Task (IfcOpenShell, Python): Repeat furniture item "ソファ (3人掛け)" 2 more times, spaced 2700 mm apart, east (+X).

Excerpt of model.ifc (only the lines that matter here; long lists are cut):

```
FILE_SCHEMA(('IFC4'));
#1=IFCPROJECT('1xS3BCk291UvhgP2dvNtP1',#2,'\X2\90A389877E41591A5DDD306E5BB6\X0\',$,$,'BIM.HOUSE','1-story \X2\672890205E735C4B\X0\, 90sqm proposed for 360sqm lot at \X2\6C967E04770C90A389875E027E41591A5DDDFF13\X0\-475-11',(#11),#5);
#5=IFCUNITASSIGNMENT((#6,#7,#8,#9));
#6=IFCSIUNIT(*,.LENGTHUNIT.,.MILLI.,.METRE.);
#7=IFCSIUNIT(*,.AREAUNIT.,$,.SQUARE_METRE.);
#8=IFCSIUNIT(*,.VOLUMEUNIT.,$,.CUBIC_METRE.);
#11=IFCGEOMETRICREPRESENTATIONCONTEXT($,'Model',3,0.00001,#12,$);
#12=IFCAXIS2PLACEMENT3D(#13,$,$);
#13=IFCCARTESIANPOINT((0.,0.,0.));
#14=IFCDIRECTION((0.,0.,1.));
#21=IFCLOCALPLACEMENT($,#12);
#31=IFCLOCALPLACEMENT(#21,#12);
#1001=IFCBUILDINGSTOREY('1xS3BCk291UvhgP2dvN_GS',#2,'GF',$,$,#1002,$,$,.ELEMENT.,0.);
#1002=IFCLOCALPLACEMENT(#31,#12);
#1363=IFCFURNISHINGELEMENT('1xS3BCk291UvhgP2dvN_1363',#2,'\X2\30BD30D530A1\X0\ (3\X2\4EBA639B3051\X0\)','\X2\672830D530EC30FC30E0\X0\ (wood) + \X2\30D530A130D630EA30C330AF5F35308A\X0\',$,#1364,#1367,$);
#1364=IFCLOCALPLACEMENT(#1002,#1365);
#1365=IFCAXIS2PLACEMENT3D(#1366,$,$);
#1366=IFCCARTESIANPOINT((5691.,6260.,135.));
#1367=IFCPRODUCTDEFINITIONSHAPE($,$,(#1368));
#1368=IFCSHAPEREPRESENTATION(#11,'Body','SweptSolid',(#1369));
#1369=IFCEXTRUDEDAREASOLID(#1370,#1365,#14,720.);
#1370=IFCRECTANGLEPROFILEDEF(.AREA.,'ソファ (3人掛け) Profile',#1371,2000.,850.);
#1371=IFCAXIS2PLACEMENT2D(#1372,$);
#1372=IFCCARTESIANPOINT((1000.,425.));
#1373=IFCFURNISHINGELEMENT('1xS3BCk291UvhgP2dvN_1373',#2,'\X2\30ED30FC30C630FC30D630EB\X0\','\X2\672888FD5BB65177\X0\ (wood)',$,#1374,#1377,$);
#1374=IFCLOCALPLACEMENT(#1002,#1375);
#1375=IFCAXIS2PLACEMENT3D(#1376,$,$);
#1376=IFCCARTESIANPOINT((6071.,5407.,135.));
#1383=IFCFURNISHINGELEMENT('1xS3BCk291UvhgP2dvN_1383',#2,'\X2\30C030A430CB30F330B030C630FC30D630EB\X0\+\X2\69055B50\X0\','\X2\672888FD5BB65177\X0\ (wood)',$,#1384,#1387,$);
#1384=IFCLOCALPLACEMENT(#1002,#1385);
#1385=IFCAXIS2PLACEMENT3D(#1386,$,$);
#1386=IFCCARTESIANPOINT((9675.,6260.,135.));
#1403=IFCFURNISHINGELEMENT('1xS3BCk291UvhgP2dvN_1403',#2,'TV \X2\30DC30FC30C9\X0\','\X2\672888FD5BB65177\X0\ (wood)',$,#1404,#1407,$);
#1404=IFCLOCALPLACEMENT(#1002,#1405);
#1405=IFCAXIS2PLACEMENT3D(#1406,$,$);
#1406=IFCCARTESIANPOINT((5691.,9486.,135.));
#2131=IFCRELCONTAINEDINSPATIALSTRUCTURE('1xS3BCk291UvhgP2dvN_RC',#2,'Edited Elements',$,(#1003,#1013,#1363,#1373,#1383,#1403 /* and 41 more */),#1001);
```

```python
import numpy as np
import ifcopenshell
import ifcopenshell.api.geometry
import ifcopenshell.api.root
import ifcopenshell.util.element
import ifcopenshell.util.placement

model = ifcopenshell.open("model.ifc")


def reuse_history(source, copy):
    """copy_class also copies each property set's owner history, people and application; keep the originals."""
    for rel in copy.IsDefinedBy:
        if rel.is_a("IfcRelDefinesByProperties") and (history := rel.RelatingPropertyDefinition.OwnerHistory):
            rel.RelatingPropertyDefinition.OwnerHistory = source.OwnerHistory
            ifcopenshell.util.element.remove_deep2(model, history)


source = model.by_guid("1xS3BCk291UvhgP2dvN_1363")
base = ifcopenshell.util.placement.get_local_placement(source.ObjectPlacement)
step = np.array([1.0, 0.0, 0.0]) * 2700.0

for i in range(1, 3):
    copy = ifcopenshell.api.root.copy_class(model, product=source)
    copy.Representation = ifcopenshell.util.element.copy_deep(
        model, source.Representation, exclude=["IfcGeometricRepresentationContext", "IfcRepresentationMap"]
    )
    reuse_history(source, copy)
    matrix = base.copy()
    matrix[:3, 3] += i * step
    print("added at", matrix[:3, 3].round(3) + 0.0)
    ifcopenshell.api.geometry.edit_object_placement(model, product=copy, matrix=matrix, is_si=False)

model.write("model_rev.ifc")
```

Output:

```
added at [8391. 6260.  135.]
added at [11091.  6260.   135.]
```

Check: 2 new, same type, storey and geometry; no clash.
